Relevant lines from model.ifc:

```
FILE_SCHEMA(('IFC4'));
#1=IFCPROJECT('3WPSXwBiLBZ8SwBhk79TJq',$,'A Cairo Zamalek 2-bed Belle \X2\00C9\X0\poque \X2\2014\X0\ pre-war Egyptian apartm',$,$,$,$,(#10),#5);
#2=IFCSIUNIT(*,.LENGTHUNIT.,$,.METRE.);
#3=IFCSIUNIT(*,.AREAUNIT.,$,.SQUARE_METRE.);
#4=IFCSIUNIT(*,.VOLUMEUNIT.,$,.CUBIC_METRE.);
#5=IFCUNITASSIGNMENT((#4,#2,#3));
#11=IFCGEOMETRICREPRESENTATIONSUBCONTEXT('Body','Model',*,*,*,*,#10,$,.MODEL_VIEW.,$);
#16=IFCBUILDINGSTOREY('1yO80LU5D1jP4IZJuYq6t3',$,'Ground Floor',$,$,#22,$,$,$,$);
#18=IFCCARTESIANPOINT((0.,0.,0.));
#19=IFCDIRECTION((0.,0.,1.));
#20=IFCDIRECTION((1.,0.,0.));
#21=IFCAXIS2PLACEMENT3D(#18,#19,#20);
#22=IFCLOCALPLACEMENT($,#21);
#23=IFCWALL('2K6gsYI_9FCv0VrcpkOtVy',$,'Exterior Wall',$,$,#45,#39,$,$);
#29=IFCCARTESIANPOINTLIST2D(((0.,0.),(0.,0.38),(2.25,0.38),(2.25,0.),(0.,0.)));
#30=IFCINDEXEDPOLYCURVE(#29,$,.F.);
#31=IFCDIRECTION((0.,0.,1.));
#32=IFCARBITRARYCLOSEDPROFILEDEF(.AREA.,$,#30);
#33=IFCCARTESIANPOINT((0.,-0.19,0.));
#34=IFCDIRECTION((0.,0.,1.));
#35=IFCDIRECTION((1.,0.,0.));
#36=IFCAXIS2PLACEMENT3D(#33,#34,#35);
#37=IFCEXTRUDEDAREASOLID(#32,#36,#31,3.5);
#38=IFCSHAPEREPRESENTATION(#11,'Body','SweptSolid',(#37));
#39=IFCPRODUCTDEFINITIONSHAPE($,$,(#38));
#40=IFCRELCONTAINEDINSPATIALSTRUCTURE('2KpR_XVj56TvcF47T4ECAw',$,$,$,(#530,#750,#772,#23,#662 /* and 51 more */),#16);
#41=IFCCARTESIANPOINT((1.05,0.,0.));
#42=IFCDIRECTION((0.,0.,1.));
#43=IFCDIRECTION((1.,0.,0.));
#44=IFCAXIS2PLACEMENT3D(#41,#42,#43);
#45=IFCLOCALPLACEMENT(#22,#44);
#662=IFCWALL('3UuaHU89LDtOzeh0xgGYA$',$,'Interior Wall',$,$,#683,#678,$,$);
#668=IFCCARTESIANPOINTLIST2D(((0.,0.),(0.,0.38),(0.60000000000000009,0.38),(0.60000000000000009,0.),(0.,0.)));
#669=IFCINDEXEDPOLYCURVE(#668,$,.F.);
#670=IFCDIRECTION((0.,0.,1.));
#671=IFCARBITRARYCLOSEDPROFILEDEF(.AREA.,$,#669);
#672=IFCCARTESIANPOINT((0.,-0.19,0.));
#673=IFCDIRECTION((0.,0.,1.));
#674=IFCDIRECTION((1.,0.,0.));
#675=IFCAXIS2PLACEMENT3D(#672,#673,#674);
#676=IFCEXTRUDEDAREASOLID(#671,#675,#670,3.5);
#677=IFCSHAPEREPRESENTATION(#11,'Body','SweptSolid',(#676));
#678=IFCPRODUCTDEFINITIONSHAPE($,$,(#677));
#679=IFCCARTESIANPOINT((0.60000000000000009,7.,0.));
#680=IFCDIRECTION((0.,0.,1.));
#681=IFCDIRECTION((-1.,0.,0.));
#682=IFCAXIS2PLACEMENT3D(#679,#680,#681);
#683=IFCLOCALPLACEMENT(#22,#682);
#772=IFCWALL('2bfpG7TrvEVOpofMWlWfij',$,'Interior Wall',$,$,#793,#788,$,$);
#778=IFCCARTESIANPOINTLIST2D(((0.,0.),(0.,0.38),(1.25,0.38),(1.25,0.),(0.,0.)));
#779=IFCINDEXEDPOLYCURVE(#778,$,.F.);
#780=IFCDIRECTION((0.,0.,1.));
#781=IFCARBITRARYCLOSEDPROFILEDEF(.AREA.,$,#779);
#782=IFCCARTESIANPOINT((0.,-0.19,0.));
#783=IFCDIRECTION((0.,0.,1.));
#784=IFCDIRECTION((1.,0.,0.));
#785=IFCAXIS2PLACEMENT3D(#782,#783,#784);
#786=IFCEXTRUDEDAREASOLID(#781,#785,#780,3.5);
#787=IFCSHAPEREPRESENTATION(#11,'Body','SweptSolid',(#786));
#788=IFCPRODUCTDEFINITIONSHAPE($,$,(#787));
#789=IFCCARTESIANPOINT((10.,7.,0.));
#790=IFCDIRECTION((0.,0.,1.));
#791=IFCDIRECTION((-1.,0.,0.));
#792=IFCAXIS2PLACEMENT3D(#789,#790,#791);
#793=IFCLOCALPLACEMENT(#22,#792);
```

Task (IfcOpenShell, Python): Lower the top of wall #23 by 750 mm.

```python
import ifcopenshell
import ifcopenshell.geom
import ifcopenshell.util.representation
import ifcopenshell.util.shape
import ifcopenshell.util.unit

model = ifcopenshell.open("model.ifc")
unit_scale = ifcopenshell.util.unit.calculate_unit_scale(model)
settings = ifcopenshell.geom.settings()


def volume(element):
    """Net volume in cubic metres, openings subtracted."""
    shape = ifcopenshell.geom.create_shape(settings, element)
    return ifcopenshell.util.shape.get_volume(shape.geometry)


wall = model.by_guid("2K6gsYI_9FCv0VrcpkOtVy")
before = volume(wall)

body = ifcopenshell.util.representation.get_representation(wall, "Model", "Body")
solid = body.Items[0]
old_height = solid.Depth
solid.Depth -= 0.75 / unit_scale
after = volume(wall)

print(f"height {old_height:g} -> {solid.Depth:g}, volume {before:.3f} -> {after:.3f} m3")

model.write("model_edited.ifc")
```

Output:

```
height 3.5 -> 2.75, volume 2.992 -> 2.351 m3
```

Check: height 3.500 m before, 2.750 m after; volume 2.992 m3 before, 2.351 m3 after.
